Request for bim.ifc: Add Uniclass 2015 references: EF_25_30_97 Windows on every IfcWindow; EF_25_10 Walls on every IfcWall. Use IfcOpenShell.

First a look at what the model holds.

```python
import ifcopenshell

model = ifcopenshell.open("bim.ifc")
print(model.schema)
print("classifications:", [c.Name for c in model.by_type("IfcClassification")])
for ifc_class in ("IfcDoor", "IfcRoof", "IfcStair", "IfcWall", "IfcWindow"):
    print(ifc_class, len(model.by_type(ifc_class)))
```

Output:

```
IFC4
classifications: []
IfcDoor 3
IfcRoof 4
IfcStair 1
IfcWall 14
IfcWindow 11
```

```python
import ifcopenshell
import ifcopenshell.api.classification

model = ifcopenshell.open("bim.ifc")

system = ifcopenshell.api.classification.add_classification(model, classification="Uniclass 2015")

codes = {
    "IfcWindow": ("EF_25_30_97", "Windows"),
    "IfcWall": ("EF_25_10", "Walls"),
}
for ifc_class, (code, name) in codes.items():
    products = model.by_type(ifc_class)
    ifcopenshell.api.classification.add_reference(
        model, products=products, classification=system, identification=code, name=name
    )
    print(code, len(products))

model.write("bim_rev.ifc")
```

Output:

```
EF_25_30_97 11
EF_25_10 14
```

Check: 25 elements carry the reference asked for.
